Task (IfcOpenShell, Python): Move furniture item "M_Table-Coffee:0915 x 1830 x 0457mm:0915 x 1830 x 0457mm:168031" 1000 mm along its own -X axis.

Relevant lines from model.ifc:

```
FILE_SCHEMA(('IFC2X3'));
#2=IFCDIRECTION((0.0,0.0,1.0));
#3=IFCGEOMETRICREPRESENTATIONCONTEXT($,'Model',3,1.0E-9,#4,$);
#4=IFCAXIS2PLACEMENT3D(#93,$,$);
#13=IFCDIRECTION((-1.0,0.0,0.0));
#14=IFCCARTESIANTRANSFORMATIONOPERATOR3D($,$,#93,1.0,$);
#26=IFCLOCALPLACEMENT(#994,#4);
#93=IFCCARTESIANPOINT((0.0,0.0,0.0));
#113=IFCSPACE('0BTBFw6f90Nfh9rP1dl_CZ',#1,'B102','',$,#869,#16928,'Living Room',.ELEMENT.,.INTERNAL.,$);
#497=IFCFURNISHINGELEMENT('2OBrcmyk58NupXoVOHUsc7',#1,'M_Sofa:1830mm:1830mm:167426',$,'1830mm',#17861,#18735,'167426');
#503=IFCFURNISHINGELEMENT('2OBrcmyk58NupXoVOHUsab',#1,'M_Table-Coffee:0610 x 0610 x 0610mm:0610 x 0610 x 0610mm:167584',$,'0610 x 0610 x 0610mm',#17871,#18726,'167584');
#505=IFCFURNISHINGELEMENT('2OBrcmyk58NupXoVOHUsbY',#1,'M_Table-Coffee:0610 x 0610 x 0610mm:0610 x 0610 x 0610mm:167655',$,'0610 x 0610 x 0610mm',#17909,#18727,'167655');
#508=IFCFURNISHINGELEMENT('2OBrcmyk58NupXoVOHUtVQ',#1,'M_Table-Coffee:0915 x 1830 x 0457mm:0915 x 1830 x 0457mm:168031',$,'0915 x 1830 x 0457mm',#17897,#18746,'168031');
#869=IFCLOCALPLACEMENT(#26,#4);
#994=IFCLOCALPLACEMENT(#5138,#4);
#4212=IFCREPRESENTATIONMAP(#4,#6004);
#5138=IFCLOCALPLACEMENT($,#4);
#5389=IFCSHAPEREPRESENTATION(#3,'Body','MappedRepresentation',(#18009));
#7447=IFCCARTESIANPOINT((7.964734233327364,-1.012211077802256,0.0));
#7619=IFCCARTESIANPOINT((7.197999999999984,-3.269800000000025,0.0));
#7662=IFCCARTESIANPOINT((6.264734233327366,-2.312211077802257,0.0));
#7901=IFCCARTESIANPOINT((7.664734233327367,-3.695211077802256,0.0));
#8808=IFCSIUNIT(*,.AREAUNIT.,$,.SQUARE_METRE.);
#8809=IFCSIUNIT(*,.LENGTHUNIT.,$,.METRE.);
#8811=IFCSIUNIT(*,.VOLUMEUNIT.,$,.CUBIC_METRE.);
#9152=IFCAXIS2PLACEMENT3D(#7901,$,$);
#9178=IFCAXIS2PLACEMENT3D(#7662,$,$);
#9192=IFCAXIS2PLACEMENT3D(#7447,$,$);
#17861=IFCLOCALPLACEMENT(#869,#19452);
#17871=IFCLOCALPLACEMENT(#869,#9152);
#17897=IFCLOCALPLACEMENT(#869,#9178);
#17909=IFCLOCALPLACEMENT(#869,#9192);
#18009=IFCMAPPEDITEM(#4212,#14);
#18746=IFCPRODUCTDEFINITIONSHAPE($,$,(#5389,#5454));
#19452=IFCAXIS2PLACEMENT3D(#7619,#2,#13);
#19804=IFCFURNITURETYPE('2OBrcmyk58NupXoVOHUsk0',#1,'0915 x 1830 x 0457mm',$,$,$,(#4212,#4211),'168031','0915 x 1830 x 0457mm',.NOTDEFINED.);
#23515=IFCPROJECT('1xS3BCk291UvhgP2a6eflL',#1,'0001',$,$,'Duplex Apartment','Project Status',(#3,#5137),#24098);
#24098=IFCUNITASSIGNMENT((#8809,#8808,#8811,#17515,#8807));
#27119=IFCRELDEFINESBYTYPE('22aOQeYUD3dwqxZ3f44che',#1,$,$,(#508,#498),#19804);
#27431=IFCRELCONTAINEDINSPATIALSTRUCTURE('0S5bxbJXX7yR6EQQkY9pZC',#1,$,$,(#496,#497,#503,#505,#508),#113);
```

```python
import ifcopenshell
import ifcopenshell.api.geometry
import ifcopenshell.util.placement
import ifcopenshell.util.unit

model = ifcopenshell.open("model.ifc")
unit_scale = ifcopenshell.util.unit.calculate_unit_scale(model)

item = model.by_id(508)
matrix = ifcopenshell.util.placement.get_local_placement(item.ObjectPlacement)
matrix[:3, 3] -= matrix[:3, 0] * 1 / unit_scale
ifcopenshell.api.geometry.edit_object_placement(model, product=item, matrix=matrix, is_si=False)

print(ifcopenshell.util.placement.get_local_placement(item.ObjectPlacement).round(3) + 0.0)

model.write("model_updated.ifc")
```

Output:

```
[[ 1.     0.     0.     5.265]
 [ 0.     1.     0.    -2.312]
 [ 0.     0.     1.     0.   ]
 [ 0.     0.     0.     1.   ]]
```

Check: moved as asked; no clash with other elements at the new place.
